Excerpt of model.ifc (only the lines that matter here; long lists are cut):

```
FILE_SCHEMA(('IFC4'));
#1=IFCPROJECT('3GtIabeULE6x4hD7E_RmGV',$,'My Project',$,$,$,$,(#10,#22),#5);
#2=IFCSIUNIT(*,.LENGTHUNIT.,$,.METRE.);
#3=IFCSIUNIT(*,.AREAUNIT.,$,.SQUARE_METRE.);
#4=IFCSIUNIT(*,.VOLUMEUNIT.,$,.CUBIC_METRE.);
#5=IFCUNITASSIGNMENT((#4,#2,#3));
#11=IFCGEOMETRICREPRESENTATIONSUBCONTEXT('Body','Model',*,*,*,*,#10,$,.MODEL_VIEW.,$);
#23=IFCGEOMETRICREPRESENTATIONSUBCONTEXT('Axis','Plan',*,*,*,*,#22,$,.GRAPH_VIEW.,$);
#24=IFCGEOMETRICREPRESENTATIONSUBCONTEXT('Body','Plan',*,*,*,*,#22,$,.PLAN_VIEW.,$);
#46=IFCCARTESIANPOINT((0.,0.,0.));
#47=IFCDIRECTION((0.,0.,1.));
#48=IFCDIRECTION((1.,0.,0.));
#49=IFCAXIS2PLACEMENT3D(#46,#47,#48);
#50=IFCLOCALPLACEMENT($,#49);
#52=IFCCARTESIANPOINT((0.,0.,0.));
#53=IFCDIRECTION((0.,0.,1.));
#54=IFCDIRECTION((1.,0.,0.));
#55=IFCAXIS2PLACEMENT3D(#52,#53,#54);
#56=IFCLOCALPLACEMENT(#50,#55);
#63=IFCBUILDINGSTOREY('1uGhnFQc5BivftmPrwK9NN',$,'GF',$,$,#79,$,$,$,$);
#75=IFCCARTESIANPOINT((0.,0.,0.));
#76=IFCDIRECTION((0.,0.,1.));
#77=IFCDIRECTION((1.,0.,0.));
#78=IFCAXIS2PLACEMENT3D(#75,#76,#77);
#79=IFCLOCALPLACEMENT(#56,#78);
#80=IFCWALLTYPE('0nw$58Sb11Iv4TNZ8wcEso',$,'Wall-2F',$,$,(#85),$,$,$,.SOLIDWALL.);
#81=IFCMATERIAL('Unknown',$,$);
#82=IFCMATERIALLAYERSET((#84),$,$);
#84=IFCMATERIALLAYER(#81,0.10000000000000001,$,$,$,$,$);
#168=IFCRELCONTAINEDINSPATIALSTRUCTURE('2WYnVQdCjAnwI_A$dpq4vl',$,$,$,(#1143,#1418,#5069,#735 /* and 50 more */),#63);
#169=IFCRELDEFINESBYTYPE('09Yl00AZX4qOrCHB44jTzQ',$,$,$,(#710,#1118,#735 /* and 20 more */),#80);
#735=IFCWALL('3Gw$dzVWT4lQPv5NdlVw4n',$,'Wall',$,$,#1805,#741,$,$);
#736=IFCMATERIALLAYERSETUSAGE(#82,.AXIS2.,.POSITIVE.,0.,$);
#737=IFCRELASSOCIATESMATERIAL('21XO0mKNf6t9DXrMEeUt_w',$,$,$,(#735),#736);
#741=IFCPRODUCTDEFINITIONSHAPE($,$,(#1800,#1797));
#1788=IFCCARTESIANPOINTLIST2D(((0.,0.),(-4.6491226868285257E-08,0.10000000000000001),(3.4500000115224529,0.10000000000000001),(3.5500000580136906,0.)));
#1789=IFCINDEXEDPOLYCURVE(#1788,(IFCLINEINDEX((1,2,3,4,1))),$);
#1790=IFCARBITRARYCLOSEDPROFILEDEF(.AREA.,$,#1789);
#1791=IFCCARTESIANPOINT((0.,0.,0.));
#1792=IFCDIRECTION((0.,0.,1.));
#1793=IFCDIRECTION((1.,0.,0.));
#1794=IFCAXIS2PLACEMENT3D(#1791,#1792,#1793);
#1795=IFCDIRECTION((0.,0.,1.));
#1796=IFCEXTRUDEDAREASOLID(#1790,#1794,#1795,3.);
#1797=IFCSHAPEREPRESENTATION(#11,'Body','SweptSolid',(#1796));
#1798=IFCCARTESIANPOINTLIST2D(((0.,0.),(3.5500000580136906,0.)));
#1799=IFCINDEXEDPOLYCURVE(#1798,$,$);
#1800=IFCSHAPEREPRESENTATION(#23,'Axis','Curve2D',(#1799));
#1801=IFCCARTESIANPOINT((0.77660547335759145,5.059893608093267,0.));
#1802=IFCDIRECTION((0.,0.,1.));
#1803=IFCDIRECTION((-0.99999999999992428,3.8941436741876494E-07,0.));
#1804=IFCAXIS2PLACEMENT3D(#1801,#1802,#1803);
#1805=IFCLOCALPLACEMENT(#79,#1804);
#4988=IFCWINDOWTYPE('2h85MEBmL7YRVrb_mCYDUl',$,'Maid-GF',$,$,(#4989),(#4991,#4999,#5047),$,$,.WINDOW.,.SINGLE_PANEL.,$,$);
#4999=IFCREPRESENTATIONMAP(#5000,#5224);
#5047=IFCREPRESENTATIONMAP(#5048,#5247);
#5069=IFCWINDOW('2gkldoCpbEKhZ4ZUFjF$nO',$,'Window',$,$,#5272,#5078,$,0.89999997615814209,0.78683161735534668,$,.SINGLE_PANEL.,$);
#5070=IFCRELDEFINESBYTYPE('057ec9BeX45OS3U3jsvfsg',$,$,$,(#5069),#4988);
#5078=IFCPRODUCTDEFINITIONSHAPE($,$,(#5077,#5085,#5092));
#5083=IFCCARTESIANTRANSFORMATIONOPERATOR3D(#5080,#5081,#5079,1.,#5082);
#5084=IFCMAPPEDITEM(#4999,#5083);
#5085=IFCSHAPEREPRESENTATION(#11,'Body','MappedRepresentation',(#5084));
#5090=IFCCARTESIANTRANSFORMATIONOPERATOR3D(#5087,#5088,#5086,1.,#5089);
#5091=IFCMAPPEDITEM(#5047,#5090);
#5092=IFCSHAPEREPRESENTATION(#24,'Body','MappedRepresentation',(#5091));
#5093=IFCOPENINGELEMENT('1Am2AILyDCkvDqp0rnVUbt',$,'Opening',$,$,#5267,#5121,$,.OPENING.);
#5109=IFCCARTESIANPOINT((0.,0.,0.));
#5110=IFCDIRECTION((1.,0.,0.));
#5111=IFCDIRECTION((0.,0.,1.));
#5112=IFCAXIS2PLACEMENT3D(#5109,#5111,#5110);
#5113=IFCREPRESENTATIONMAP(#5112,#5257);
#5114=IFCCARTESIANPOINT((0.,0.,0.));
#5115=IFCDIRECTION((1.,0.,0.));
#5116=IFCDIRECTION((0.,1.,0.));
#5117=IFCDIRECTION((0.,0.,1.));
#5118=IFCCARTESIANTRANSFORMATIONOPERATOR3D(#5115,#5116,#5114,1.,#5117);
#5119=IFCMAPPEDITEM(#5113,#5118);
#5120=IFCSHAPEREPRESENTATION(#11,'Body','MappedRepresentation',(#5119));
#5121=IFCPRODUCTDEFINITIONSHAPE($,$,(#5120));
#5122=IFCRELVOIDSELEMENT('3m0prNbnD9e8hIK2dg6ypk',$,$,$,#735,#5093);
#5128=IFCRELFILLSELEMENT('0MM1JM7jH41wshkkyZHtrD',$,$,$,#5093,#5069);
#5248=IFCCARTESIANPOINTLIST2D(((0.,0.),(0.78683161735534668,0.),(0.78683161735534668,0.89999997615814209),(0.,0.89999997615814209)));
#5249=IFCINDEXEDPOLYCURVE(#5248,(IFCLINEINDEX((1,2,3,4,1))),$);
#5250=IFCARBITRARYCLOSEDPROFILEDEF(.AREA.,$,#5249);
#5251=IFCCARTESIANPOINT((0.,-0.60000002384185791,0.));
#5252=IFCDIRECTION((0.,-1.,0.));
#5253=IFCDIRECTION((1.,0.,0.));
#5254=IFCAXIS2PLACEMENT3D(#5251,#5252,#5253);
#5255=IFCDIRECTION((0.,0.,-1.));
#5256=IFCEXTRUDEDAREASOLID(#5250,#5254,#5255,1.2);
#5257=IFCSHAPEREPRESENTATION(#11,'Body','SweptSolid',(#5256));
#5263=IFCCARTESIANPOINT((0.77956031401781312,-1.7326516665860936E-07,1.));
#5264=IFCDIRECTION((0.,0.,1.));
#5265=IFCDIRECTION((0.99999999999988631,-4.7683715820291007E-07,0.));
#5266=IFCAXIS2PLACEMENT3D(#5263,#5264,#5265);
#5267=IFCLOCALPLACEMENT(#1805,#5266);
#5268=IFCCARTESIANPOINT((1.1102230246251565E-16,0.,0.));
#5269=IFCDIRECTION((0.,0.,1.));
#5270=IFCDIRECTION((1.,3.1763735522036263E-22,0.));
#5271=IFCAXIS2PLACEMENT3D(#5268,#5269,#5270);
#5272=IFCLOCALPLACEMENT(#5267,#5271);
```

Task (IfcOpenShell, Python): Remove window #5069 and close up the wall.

```python
import ifcopenshell
import ifcopenshell.api.feature
import ifcopenshell.api.root
import ifcopenshell.geom
import ifcopenshell.util.shape

model = ifcopenshell.open("model.ifc")
settings = ifcopenshell.geom.settings()


def volume(element):
    """Net volume in cubic metres, openings subtracted."""
    shape = ifcopenshell.geom.create_shape(settings, element)
    return ifcopenshell.util.shape.get_volume(shape.geometry)


window = model.by_id(5069)
opening = window.FillsVoids[0].RelatingOpeningElement
wall = opening.VoidsElements[0].RelatingBuildingElement
before = volume(wall)

ifcopenshell.api.root.remove_product(model, product=window)
ifcopenshell.api.feature.remove_feature(model, feature=opening)

after = volume(wall)

print(f"wall volume {before:.3f} -> {after:.3f} m3")

model.write("model_rev.ifc")
```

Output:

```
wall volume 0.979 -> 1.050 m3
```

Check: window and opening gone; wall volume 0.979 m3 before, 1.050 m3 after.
